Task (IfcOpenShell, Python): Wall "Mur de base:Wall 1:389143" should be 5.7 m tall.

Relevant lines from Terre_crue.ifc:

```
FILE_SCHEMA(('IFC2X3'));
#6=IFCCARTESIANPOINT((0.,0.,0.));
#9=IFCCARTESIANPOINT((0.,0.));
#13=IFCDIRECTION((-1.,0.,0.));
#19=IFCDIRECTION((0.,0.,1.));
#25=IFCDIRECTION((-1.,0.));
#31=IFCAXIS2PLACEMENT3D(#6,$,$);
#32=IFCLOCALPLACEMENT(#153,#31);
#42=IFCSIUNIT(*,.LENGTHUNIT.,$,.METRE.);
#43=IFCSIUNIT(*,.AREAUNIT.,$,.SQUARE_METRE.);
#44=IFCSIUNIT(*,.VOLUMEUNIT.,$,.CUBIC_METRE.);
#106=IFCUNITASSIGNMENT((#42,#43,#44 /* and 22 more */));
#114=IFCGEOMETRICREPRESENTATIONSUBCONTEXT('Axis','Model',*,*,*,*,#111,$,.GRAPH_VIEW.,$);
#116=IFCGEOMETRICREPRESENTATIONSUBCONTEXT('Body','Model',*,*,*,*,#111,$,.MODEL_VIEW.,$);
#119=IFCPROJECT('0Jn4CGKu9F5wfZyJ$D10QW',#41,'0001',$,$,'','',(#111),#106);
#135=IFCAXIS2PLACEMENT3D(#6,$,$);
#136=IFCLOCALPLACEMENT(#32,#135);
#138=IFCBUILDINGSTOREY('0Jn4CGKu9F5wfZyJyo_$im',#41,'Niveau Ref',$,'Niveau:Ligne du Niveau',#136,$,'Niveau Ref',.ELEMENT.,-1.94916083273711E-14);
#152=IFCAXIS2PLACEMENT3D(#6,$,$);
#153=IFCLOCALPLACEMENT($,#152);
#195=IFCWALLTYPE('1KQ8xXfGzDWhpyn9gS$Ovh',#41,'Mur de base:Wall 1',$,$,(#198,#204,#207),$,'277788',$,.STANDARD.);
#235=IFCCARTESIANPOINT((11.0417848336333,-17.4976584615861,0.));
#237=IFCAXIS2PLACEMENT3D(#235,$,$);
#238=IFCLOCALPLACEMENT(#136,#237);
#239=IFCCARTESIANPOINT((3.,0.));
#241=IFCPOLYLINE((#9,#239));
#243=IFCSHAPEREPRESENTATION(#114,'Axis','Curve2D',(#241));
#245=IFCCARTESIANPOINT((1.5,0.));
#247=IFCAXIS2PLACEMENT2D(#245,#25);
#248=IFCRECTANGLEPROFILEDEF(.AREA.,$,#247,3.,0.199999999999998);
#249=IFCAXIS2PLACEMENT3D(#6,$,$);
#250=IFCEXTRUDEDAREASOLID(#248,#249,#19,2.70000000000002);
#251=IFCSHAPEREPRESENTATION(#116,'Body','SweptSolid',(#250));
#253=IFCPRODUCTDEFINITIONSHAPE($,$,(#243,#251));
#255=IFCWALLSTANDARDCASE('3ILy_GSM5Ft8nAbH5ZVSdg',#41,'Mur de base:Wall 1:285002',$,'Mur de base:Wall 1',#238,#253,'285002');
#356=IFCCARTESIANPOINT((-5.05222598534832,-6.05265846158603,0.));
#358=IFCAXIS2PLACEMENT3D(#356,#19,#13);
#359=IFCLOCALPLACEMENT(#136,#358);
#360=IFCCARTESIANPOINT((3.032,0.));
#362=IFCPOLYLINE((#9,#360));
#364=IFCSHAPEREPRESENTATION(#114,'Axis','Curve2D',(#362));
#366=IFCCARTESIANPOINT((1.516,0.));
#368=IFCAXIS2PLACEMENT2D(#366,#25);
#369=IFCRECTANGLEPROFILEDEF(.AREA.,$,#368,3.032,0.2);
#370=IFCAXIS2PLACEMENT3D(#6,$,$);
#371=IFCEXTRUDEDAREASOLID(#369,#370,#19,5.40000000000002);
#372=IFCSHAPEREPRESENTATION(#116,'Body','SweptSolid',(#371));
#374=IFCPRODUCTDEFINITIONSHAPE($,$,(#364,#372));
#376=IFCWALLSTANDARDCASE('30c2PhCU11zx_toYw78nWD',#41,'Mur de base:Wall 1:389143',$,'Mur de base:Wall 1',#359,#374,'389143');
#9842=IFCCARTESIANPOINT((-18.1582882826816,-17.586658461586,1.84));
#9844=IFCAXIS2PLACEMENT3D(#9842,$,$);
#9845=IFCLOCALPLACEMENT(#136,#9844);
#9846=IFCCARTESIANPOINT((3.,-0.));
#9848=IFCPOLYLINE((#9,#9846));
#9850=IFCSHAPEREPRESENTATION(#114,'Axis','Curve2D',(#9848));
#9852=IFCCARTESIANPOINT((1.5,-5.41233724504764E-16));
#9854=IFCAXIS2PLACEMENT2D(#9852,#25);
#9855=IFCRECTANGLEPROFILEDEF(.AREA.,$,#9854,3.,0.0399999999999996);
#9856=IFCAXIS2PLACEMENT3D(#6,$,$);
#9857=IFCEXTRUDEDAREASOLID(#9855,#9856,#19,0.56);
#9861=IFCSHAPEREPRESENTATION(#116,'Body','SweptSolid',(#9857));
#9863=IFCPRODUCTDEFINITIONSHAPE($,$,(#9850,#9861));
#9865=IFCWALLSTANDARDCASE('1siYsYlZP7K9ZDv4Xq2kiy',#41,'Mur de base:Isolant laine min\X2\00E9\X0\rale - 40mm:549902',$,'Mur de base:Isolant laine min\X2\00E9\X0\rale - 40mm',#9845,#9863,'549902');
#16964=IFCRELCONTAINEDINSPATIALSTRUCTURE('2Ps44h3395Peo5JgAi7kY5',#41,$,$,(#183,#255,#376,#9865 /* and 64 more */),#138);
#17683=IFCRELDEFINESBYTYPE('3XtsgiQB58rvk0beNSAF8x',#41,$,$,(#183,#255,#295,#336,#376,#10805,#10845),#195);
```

```python
import ifcopenshell
import ifcopenshell.geom
import ifcopenshell.util.representation
import ifcopenshell.util.shape
import ifcopenshell.util.unit

model = ifcopenshell.open("Terre_crue.ifc")
unit_scale = ifcopenshell.util.unit.calculate_unit_scale(model)
settings = ifcopenshell.geom.settings()


def volume(element):
    """Net volume in cubic metres, openings subtracted."""
    shape = ifcopenshell.geom.create_shape(settings, element)
    return ifcopenshell.util.shape.get_volume(shape.geometry)


wall = model.by_guid("30c2PhCU11zx_toYw78nWD")
before = volume(wall)

body = ifcopenshell.util.representation.get_representation(wall, "Model", "Body")
solid = body.Items[0]
old_height = solid.Depth
solid.Depth = 5.7 / unit_scale
after = volume(wall)

print(f"height {old_height:g} -> {solid.Depth:g}, volume {before:.3f} -> {after:.3f} m3")

model.write("Terre_crue_rev.ifc")
```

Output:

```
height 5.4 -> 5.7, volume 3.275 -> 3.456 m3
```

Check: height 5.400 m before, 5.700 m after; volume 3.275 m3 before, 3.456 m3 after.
